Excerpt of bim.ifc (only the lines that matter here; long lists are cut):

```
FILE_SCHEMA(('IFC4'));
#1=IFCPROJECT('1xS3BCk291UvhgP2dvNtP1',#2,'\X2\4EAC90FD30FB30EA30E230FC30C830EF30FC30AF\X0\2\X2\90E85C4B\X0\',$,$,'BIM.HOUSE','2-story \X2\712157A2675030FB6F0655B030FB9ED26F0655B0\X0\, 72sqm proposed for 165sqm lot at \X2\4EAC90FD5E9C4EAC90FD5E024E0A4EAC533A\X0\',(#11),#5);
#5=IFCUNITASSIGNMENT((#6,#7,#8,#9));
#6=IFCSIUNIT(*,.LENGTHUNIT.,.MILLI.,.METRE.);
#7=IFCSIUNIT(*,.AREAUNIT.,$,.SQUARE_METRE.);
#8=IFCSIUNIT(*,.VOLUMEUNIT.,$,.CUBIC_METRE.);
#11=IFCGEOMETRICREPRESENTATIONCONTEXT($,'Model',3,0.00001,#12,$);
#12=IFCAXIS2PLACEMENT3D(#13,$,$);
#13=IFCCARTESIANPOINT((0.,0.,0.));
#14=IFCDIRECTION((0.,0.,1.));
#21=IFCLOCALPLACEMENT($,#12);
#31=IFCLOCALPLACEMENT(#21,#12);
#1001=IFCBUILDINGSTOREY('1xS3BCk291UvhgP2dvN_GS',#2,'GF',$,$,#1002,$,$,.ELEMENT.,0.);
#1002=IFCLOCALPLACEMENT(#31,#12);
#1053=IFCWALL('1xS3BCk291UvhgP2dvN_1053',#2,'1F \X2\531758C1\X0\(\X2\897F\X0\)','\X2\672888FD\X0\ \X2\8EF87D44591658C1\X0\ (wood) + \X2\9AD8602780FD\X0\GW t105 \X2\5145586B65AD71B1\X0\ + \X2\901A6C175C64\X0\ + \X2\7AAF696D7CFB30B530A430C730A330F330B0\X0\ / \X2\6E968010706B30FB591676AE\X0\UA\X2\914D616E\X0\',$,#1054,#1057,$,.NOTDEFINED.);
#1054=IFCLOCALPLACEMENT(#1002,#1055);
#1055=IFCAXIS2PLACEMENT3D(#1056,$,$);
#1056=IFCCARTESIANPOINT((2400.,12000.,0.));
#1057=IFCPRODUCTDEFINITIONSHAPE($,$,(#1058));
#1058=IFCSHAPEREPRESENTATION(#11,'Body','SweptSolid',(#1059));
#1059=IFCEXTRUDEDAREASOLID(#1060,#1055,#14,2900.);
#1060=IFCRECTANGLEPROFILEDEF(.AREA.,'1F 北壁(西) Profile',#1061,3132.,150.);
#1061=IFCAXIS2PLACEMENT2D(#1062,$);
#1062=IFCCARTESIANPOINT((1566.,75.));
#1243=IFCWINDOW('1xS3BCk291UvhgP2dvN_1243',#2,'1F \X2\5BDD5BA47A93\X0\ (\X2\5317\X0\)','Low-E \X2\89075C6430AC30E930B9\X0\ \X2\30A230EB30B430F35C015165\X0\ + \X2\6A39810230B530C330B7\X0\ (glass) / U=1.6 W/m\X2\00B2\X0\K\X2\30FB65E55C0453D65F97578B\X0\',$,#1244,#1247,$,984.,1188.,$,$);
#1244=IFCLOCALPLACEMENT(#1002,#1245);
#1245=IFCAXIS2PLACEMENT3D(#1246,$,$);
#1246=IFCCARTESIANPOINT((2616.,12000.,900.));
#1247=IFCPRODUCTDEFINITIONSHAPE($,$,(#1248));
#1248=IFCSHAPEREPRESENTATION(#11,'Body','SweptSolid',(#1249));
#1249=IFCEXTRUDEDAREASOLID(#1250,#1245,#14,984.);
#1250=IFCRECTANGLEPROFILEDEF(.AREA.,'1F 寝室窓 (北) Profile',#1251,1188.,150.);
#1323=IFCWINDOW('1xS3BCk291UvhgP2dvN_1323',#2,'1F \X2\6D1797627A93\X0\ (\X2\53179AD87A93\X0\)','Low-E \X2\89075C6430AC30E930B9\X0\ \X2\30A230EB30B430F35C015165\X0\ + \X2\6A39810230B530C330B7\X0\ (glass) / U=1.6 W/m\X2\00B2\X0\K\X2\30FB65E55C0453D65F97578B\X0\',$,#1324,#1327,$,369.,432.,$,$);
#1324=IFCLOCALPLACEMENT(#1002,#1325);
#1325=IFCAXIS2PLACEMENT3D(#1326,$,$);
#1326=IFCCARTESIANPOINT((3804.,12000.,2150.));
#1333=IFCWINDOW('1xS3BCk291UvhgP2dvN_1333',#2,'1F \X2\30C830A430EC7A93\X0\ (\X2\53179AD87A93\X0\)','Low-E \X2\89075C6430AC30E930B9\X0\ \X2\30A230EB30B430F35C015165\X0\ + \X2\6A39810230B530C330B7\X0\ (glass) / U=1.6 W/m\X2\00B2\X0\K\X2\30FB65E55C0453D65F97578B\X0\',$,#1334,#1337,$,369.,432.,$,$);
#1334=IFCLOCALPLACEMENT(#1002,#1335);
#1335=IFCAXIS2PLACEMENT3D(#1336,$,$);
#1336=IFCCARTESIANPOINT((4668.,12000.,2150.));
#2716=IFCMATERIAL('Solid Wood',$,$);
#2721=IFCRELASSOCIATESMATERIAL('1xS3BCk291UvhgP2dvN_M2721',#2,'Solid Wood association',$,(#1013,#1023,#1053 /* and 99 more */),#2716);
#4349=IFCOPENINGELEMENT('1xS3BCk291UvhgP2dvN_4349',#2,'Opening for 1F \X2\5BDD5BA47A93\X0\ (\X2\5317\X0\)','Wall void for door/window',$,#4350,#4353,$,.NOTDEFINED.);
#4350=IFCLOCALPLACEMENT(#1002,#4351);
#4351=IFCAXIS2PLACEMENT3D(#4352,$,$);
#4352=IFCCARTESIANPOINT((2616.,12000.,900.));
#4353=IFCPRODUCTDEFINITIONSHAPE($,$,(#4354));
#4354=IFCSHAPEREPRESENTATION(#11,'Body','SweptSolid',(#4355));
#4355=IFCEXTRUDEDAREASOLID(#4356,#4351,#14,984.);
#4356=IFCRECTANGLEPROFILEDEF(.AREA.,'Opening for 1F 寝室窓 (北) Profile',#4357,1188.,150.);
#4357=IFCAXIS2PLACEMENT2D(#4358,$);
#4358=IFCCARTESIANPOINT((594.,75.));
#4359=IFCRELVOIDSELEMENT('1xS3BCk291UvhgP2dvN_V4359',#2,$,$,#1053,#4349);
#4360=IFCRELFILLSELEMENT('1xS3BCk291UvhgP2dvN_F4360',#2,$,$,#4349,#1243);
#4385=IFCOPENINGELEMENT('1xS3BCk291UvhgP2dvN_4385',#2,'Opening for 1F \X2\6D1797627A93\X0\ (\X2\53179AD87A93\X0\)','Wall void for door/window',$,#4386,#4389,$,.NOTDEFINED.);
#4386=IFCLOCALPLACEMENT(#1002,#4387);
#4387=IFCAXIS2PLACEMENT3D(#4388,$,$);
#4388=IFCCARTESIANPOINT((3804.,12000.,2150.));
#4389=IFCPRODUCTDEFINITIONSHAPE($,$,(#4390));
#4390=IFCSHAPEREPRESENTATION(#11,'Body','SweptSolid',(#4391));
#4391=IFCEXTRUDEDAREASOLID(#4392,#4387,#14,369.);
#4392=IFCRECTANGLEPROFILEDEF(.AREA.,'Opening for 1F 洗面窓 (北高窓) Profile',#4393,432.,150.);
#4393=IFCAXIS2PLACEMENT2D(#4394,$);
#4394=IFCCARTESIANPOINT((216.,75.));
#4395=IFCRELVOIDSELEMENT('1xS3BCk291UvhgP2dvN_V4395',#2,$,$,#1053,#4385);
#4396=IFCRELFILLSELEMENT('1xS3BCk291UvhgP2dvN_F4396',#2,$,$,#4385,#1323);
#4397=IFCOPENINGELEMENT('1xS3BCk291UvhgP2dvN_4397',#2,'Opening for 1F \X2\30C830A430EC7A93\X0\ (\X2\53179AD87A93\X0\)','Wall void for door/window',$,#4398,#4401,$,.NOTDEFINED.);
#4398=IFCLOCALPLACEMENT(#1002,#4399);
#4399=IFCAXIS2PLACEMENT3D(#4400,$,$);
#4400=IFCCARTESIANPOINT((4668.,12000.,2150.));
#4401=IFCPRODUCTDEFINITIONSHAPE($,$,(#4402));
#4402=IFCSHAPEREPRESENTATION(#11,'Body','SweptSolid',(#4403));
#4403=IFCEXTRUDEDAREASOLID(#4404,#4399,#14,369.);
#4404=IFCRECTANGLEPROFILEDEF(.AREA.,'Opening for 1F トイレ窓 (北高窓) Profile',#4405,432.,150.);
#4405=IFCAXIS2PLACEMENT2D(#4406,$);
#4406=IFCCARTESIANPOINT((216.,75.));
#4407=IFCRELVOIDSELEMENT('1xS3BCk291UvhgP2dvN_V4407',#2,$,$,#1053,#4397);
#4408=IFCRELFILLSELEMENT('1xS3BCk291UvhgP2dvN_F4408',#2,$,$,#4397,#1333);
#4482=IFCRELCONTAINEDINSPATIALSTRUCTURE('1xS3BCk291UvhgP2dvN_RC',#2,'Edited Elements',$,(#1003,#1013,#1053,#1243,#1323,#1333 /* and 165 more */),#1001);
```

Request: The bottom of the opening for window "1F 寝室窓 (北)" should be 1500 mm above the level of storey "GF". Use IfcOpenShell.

```python
import numpy as np
import ifcopenshell
import ifcopenshell.api.geometry
import ifcopenshell.geom
import ifcopenshell.util.element
import ifcopenshell.util.placement
import ifcopenshell.util.shape
import ifcopenshell.util.unit

model = ifcopenshell.open("bim.ifc")
unit_scale = ifcopenshell.util.unit.calculate_unit_scale(model)

window = model.by_guid("1xS3BCk291UvhgP2dvN_1243")
opening = window.FillsVoids[0].RelatingOpeningElement
storey = ifcopenshell.util.element.get_container(window, ifc_class="IfcBuildingStorey")
level = ifcopenshell.util.placement.get_local_placement(storey.ObjectPlacement)[2, 3]

# The opening's origin need not be at the sill, so measure its lowest point.
shape = ifcopenshell.geom.create_shape(ifcopenshell.geom.settings(), opening)
bottom = ifcopenshell.util.shape.get_shape_bottom_elevation(shape, shape.geometry) / unit_scale
dz = level + 1500.0 - bottom

shift = np.array([0.0, 0.0, dz])
# The window is not placed relative to its opening, so move both.
for product in (opening, window):
    matrix = ifcopenshell.util.placement.get_local_placement(product.ObjectPlacement)
    matrix[:3, 3] += shift
    ifcopenshell.api.geometry.edit_object_placement(model, product=product, matrix=matrix, is_si=False)

print(f"moved by {dz * unit_scale:+.3f} m")

model.write("bim_v2.ifc")
```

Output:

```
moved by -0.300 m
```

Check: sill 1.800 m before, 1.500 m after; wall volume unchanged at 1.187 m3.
